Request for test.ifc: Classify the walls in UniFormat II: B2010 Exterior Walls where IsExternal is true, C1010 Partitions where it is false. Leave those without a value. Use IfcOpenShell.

First a look at what the model holds.

```python
import ifcopenshell
import ifcopenshell.util.element

model = ifcopenshell.open("test.ifc")
print(model.schema)
print("classifications:", [c.Name for c in model.by_type("IfcClassification")])
values = [ifcopenshell.util.element.get_pset(e, "Pset_WallCommon", "IsExternal") for e in model.by_type("IfcWall")]
for value in (True, False, None):
    print("IsExternal", value, values.count(value))
```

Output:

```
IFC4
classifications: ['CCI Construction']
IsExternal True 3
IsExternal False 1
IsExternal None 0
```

```python
import ifcopenshell
import ifcopenshell.api.classification
import ifcopenshell.util.element

model = ifcopenshell.open("test.ifc")

system = ifcopenshell.api.classification.add_classification(model, classification="UniFormat II")

walls = model.by_type("IfcWall")
external = {e: ifcopenshell.util.element.get_pset(e, "Pset_WallCommon", "IsExternal") for e in walls}
for flag, code, name in ((True, "B2010", "Exterior Walls"), (False, "C1010", "Partitions")):
    products = [e for e in walls if external[e] is flag]
    ifcopenshell.api.classification.add_reference(
        model, products=products, classification=system, identification=code, name=name
    )
    print(code, len(products))

model.write("test_rev.ifc")
```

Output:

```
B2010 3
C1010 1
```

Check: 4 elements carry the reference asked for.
